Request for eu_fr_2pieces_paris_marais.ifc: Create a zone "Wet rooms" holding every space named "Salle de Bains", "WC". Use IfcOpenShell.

First a look at what the model holds.

```python
import ifcopenshell

model = ifcopenshell.open("eu_fr_2pieces_paris_marais.ifc")
print(model.schema)
seen = {}
for space in model.by_type("IfcSpace"):
    seen[space.LongName] = seen.get(space.LongName, 0) + 1
for name, count in sorted(seen.items(), key=str):
    print(count, "x", name)
print("zones:", [z.Name for z in model.by_type("IfcZone")][:20])
```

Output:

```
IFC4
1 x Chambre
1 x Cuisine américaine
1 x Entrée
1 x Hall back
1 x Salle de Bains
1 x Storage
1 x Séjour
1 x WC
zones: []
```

```python
import ifcopenshell
import ifcopenshell.api.group
import ifcopenshell.api.root

model = ifcopenshell.open("eu_fr_2pieces_paris_marais.ifc")

names = {"Salle de Bains", "WC"}
spaces = [s for s in model.by_type("IfcSpace") if s.LongName in names]

zone = ifcopenshell.api.root.create_entity(model, ifc_class="IfcZone", name="Wet rooms")
ifcopenshell.api.group.assign_group(model, products=spaces, group=zone)
print(len(spaces), "spaces in", zone.Name)

model.write("eu_fr_2pieces_paris_marais_rev.ifc")
```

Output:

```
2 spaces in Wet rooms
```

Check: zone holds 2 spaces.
